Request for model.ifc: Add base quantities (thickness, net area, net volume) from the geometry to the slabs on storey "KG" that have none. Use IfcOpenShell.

First a look at what the model holds.

```python
import ifcopenshell
import ifcopenshell.util.element
import ifcopenshell.util.unit

model = ifcopenshell.open("model.ifc")
print(model.schema)
for unit_type in ("LENGTHUNIT", "AREAUNIT", "VOLUMEUNIT"):
    print(unit_type, ifcopenshell.util.unit.calculate_unit_scale(model, unit_type))
storey = next(s for s in model.by_type("IfcBuildingStorey") if s.Name == "KG")
slabs = [e for e in ifcopenshell.util.element.get_decomposition(storey) if e.is_a("IfcSlab")]
for e in sorted(slabs, key=lambda e: e.id()):
    print(e.id(), e.is_a(), e.Name, list(ifcopenshell.util.element.get_psets(e, qtos_only=True)), sep=" | ")
```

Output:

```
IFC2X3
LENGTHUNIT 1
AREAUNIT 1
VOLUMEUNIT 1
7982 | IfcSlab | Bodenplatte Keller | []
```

```python
import ifcopenshell
import ifcopenshell.api.pset
import ifcopenshell.geom
import ifcopenshell.util.element
import ifcopenshell.util.shape
import ifcopenshell.util.unit

model = ifcopenshell.open("model.ifc")
unit_scale = ifcopenshell.util.unit.calculate_unit_scale(model)
area_scale = ifcopenshell.util.unit.calculate_unit_scale(model, "AREAUNIT")
volume_scale = ifcopenshell.util.unit.calculate_unit_scale(model, "VOLUMEUNIT")
settings = ifcopenshell.geom.settings()

storey = next(s for s in model.by_type("IfcBuildingStorey") if s.Name == "KG")
slabs = [e for e in ifcopenshell.util.element.get_decomposition(storey) if e.is_a("IfcSlab")]

for e in sorted(slabs, key=lambda e: e.id()):
    if ifcopenshell.util.element.get_psets(e, qtos_only=True, should_inherit=False):
        continue
    # Geometry comes back in metres, in the element's own axes.
    shape = ifcopenshell.geom.create_shape(settings, e)
    values = {
        "Width": ifcopenshell.util.shape.get_z(shape.geometry) / unit_scale,
        "NetArea": ifcopenshell.util.shape.get_footprint_area(shape.geometry) / area_scale,
        "NetVolume": ifcopenshell.util.shape.get_volume(shape.geometry) / volume_scale,
    }
    qto = ifcopenshell.api.pset.add_qto(model, product=e, name="BaseQuantities")
    ifcopenshell.api.pset.edit_qto(model, qto=qto, properties=values)
    print(e.id(), {k: round(v, 3) for k, v in values.items()})

model.write("model_v2.ifc")
```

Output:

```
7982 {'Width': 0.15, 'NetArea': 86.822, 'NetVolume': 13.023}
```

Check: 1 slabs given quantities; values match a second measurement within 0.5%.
